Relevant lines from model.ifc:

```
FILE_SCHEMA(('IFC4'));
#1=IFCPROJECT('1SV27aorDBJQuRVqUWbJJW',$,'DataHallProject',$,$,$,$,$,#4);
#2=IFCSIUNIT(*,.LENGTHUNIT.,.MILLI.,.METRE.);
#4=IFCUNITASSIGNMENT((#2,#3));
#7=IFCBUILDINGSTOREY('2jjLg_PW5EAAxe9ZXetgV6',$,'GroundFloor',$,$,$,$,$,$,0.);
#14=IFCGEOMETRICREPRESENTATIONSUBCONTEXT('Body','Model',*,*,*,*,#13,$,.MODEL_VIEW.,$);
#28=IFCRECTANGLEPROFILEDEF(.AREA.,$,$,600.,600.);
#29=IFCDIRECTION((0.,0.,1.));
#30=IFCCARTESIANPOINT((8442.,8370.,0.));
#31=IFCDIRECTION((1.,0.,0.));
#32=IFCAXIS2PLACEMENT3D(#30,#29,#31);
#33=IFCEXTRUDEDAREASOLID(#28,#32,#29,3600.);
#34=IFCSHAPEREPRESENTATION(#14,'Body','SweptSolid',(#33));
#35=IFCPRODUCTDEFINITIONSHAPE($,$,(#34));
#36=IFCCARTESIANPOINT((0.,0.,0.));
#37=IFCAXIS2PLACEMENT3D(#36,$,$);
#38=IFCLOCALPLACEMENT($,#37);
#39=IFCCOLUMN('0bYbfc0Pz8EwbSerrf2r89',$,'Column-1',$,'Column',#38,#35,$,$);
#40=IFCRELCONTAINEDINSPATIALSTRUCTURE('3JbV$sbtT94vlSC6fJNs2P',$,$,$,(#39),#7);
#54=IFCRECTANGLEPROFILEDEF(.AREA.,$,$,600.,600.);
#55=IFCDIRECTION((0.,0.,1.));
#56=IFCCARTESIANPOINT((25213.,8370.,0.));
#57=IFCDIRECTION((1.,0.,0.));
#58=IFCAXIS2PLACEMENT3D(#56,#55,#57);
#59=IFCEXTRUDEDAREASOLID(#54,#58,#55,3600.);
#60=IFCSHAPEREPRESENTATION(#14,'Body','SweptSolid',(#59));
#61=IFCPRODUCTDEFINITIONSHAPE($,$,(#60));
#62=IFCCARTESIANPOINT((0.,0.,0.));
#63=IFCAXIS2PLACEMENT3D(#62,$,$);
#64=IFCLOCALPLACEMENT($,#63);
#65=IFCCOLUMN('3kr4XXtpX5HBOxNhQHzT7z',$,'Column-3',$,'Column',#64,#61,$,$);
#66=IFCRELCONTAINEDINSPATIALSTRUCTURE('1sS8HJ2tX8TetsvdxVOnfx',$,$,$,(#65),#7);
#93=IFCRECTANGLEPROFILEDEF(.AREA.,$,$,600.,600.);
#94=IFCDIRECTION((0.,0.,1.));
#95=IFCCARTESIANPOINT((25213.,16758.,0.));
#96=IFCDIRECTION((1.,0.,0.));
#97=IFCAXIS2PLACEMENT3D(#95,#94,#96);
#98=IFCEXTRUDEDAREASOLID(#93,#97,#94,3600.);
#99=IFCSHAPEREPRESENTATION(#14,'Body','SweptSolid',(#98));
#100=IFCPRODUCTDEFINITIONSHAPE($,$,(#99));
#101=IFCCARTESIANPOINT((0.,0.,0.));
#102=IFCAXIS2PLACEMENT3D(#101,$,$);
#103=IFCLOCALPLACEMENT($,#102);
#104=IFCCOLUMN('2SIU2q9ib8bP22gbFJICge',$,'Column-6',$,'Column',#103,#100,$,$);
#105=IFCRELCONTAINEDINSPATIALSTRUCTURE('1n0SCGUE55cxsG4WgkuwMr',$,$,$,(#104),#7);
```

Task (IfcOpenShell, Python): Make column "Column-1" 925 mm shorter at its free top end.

```python
import ifcopenshell
import ifcopenshell.util.representation
import ifcopenshell.util.unit

model = ifcopenshell.open("model.ifc")
unit_scale = ifcopenshell.util.unit.calculate_unit_scale(model)

member = model.by_guid("0bYbfc0Pz8EwbSerrf2r89")
change = -0.925 / unit_scale

# The extrusion runs towards the end named, so only its depth changes.
body = ifcopenshell.util.representation.get_representation(member, "Model", "Body")
solid = body.Items[0]
old_length = solid.Depth
solid.Depth += change

print(f"length {old_length:g} -> {solid.Depth:g}")

model.write("model_v2.ifc")
```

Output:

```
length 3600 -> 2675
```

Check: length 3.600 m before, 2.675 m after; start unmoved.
